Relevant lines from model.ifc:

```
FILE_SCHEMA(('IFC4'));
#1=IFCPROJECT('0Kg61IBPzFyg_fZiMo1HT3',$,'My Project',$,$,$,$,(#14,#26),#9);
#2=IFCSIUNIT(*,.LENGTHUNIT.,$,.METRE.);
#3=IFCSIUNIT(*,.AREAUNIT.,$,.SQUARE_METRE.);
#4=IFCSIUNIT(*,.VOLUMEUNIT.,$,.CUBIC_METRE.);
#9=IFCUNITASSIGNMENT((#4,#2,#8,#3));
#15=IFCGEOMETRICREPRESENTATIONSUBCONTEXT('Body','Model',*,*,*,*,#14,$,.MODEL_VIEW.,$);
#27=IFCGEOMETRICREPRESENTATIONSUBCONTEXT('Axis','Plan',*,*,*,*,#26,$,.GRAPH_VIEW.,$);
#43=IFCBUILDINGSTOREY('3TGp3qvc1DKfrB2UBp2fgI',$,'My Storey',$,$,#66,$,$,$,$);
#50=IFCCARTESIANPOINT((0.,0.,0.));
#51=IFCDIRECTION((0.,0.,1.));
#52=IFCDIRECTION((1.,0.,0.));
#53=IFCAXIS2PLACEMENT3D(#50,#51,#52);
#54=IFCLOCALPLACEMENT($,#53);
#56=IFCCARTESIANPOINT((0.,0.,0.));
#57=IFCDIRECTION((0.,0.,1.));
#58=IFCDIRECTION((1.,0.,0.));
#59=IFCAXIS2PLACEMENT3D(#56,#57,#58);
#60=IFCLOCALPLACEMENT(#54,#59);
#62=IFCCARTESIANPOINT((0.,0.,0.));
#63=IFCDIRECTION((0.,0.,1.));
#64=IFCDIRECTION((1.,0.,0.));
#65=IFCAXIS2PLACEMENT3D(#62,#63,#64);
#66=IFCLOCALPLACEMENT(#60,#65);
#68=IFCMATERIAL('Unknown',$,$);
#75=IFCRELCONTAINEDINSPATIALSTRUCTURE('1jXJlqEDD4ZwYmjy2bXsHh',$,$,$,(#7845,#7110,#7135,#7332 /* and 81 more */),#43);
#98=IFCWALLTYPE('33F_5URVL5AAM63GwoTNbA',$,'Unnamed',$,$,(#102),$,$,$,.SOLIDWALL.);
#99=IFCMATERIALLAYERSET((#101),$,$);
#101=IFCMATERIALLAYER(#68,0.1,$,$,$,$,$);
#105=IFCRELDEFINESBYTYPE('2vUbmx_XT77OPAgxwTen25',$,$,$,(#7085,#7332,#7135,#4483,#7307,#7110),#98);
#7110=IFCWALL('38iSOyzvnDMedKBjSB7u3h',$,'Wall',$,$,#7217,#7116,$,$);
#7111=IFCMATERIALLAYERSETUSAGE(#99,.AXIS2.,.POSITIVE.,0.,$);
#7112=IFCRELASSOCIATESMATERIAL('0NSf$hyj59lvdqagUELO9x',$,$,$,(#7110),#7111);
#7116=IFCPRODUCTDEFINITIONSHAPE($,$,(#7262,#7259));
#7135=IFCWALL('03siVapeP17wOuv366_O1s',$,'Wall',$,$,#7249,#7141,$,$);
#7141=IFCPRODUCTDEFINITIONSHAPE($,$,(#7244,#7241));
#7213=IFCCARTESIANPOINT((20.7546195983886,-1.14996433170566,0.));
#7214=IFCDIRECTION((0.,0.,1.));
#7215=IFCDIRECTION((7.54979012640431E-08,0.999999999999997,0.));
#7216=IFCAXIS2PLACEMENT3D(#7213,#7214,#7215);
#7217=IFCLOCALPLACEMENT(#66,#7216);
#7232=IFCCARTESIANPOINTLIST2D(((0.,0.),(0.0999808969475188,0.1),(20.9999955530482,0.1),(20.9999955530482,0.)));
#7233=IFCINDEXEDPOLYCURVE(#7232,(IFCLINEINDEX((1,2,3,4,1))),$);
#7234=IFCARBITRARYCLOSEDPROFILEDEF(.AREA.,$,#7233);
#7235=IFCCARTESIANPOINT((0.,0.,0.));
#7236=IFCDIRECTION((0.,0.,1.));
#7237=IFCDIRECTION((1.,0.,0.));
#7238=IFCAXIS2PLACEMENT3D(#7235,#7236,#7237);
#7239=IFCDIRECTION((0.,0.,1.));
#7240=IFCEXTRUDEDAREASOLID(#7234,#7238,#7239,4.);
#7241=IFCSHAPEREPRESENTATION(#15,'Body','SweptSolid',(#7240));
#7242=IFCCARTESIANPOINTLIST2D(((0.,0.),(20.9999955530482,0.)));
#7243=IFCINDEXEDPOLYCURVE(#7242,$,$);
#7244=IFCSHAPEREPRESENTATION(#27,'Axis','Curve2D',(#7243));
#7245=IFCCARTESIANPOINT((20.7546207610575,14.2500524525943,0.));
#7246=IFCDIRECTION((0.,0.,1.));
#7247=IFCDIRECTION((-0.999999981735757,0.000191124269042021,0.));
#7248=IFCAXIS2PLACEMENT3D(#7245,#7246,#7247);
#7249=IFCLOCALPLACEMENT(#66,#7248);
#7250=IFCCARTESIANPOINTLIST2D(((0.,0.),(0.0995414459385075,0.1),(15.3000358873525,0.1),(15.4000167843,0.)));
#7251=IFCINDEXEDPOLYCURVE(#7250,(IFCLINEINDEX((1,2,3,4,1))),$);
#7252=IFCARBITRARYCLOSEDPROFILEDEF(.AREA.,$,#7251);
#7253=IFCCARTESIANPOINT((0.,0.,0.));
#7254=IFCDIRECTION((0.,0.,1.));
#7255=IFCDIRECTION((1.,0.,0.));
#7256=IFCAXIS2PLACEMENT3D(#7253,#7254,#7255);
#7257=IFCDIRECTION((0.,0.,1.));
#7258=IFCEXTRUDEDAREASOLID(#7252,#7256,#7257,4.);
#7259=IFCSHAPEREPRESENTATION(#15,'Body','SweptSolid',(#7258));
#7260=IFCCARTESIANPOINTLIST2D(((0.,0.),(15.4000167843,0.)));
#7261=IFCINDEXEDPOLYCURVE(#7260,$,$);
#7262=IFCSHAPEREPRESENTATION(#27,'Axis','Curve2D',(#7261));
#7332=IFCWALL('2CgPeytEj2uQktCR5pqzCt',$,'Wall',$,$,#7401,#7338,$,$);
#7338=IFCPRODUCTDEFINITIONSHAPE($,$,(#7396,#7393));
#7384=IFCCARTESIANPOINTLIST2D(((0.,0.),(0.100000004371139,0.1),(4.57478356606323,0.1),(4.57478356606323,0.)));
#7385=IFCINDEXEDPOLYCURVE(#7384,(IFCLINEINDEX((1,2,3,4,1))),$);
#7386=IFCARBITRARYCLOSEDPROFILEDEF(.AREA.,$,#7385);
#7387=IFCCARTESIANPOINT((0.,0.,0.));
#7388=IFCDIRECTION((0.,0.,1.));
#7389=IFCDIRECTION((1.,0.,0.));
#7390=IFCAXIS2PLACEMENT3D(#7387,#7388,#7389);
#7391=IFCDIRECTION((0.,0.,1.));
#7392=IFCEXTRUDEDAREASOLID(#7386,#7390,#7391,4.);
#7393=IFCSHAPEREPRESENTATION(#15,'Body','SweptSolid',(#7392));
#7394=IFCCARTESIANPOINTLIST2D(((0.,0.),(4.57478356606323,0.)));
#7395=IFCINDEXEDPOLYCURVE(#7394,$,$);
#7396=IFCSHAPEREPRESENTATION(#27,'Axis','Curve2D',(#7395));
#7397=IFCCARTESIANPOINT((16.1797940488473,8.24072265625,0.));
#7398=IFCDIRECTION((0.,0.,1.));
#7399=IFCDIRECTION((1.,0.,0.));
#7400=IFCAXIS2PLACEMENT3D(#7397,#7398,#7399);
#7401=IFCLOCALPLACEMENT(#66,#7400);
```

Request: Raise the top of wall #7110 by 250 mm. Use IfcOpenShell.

```python
import ifcopenshell
import ifcopenshell.geom
import ifcopenshell.util.representation
import ifcopenshell.util.shape
import ifcopenshell.util.unit

model = ifcopenshell.open("model.ifc")
unit_scale = ifcopenshell.util.unit.calculate_unit_scale(model)
settings = ifcopenshell.geom.settings()


def volume(element):
    """Net volume in cubic metres, openings subtracted."""
    shape = ifcopenshell.geom.create_shape(settings, element)
    return ifcopenshell.util.shape.get_volume(shape.geometry)


wall = model.by_id(7110)
before = volume(wall)

body = ifcopenshell.util.representation.get_representation(wall, "Model", "Body")
solid = body.Items[0]
old_height = solid.Depth
solid.Depth += 0.25 / unit_scale
after = volume(wall)

print(f"height {old_height:g} -> {solid.Depth:g}, volume {before:.3f} -> {after:.3f} m3")

model.write("model_rev.ifc")
```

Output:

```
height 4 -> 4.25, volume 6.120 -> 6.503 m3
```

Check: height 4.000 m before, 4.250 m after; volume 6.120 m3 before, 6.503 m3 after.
